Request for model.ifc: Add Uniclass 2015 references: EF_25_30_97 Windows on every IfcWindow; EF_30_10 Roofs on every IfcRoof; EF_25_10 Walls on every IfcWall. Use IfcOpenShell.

First a look at what the model holds.

```python
import ifcopenshell

model = ifcopenshell.open("model.ifc")
print(model.schema)
print("classifications:", [c.Name for c in model.by_type("IfcClassification")])
for ifc_class in ("IfcDoor", "IfcRoof", "IfcStair", "IfcWall", "IfcWindow"):
    print(ifc_class, len(model.by_type(ifc_class)))
```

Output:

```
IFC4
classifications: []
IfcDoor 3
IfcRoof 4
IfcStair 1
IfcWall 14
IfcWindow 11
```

```python
import ifcopenshell
import ifcopenshell.api.classification

model = ifcopenshell.open("model.ifc")

system = ifcopenshell.api.classification.add_classification(model, classification="Uniclass 2015")

codes = {
    "IfcWindow": ("EF_25_30_97", "Windows"),
    "IfcRoof": ("EF_30_10", "Roofs"),
    "IfcWall": ("EF_25_10", "Walls"),
}
for ifc_class, (code, name) in codes.items():
    products = model.by_type(ifc_class)
    ifcopenshell.api.classification.add_reference(
        model, products=products, classification=system, identification=code, name=name
    )
    print(code, len(products))

model.write("model_updated.ifc")
```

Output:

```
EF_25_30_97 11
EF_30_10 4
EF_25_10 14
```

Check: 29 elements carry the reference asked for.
